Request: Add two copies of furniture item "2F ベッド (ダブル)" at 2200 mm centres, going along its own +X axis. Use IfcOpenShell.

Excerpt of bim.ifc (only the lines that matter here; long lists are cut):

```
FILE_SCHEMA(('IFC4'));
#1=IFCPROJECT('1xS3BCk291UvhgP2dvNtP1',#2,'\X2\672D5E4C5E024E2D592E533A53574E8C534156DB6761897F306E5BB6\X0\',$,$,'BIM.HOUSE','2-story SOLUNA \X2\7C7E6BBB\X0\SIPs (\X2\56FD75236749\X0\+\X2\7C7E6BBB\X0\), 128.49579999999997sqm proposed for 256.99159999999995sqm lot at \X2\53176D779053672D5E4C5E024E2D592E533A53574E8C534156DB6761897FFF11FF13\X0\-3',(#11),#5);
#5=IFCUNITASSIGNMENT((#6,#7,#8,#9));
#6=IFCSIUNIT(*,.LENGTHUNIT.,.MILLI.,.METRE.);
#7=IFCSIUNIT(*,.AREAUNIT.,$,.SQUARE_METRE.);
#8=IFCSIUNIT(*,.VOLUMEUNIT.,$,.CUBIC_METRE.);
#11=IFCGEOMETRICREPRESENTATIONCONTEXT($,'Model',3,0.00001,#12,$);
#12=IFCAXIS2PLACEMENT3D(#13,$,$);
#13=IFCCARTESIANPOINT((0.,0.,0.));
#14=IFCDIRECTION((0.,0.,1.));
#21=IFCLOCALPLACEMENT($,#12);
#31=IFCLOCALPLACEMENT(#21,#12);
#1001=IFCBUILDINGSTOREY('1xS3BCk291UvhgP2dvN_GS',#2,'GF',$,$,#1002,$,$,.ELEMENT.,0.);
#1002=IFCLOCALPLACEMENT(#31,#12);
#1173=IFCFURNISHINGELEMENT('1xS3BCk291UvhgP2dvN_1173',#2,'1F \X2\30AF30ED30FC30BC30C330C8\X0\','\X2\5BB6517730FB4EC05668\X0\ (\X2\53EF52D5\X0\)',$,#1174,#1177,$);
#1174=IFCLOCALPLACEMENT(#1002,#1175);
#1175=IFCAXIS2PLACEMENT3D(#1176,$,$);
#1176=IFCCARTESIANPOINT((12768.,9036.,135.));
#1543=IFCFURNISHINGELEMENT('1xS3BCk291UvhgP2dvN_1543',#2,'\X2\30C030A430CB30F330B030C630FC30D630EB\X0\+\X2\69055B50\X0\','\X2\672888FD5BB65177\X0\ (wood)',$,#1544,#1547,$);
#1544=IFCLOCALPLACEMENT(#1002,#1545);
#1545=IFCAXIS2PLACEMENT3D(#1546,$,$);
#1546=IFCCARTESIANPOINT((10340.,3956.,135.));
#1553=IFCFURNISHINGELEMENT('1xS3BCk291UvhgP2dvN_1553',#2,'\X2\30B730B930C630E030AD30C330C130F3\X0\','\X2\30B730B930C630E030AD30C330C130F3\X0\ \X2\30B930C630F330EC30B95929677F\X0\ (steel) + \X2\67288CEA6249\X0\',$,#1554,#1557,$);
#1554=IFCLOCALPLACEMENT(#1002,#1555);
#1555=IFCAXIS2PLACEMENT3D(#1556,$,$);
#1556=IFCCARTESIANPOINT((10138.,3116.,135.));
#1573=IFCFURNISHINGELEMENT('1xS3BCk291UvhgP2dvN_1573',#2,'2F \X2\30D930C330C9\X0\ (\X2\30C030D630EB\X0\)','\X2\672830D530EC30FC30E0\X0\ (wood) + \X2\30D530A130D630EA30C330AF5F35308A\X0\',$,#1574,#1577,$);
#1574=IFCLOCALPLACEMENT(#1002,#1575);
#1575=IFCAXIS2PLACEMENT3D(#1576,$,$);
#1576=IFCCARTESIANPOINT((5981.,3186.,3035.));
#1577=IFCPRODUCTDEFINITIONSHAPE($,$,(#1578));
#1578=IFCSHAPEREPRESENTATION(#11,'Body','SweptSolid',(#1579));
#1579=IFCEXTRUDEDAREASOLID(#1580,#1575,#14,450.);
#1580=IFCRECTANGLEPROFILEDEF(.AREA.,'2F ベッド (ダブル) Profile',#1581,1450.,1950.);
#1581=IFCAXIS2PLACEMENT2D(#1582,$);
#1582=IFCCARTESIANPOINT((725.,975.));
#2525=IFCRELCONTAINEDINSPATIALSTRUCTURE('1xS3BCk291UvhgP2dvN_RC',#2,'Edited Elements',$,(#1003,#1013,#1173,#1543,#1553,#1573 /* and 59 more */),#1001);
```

```python
import ifcopenshell
import ifcopenshell.api.geometry
import ifcopenshell.api.root
import ifcopenshell.util.element
import ifcopenshell.util.placement

model = ifcopenshell.open("bim.ifc")


def reuse_history(source, copy):
    """copy_class also copies each property set's owner history, people and application; keep the originals."""
    for rel in copy.IsDefinedBy:
        if rel.is_a("IfcRelDefinesByProperties") and (history := rel.RelatingPropertyDefinition.OwnerHistory):
            rel.RelatingPropertyDefinition.OwnerHistory = source.OwnerHistory
            ifcopenshell.util.element.remove_deep2(model, history)


source = model.by_id(1573)
base = ifcopenshell.util.placement.get_local_placement(source.ObjectPlacement)
step = base[:3, 0] * 2200.0

for i in range(1, 3):
    copy = ifcopenshell.api.root.copy_class(model, product=source)
    copy.Representation = ifcopenshell.util.element.copy_deep(
        model, source.Representation, exclude=["IfcGeometricRepresentationContext", "IfcRepresentationMap"]
    )
    reuse_history(source, copy)
    matrix = base.copy()
    matrix[:3, 3] += i * step
    print("added at", matrix[:3, 3].round(3) + 0.0)
    ifcopenshell.api.geometry.edit_object_placement(model, product=copy, matrix=matrix, is_si=False)

model.write("bim_v2.ifc")
```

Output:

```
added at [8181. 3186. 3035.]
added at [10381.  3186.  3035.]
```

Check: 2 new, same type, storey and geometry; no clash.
